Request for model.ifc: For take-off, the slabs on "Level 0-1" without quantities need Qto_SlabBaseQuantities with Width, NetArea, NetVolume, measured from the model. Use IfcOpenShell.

First a look at what the model holds.

```python
import ifcopenshell
import ifcopenshell.util.element
import ifcopenshell.util.unit

model = ifcopenshell.open("model.ifc")
print(model.schema)
for unit_type in ("LENGTHUNIT", "AREAUNIT", "VOLUMEUNIT"):
    print(unit_type, ifcopenshell.util.unit.calculate_unit_scale(model, unit_type))
storey = next(s for s in model.by_type("IfcBuildingStorey") if s.Name == "Level 0-1")
slabs = [e for e in ifcopenshell.util.element.get_decomposition(storey) if e.is_a("IfcSlab")]
for e in sorted(slabs, key=lambda e: e.id()):
    print(e.id(), e.is_a(), e.Name, list(ifcopenshell.util.element.get_psets(e, qtos_only=True)), sep=" | ")
```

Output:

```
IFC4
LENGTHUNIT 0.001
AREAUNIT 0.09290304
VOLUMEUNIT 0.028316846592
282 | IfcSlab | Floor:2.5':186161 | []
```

```python
import ifcopenshell
import ifcopenshell.api.pset
import ifcopenshell.geom
import ifcopenshell.util.element
import ifcopenshell.util.shape
import ifcopenshell.util.unit

model = ifcopenshell.open("model.ifc")
unit_scale = ifcopenshell.util.unit.calculate_unit_scale(model)
area_scale = ifcopenshell.util.unit.calculate_unit_scale(model, "AREAUNIT")
volume_scale = ifcopenshell.util.unit.calculate_unit_scale(model, "VOLUMEUNIT")
settings = ifcopenshell.geom.settings()

storey = next(s for s in model.by_type("IfcBuildingStorey") if s.Name == "Level 0-1")
slabs = [e for e in ifcopenshell.util.element.get_decomposition(storey) if e.is_a("IfcSlab")]

for e in sorted(slabs, key=lambda e: e.id()):
    if ifcopenshell.util.element.get_psets(e, qtos_only=True, should_inherit=False):
        continue
    # Geometry comes back in metres, in the element's own axes.
    shape = ifcopenshell.geom.create_shape(settings, e)
    values = {
        "Width": ifcopenshell.util.shape.get_z(shape.geometry) / unit_scale,
        "NetArea": ifcopenshell.util.shape.get_footprint_area(shape.geometry) / area_scale,
        "NetVolume": ifcopenshell.util.shape.get_volume(shape.geometry) / volume_scale,
    }
    qto = ifcopenshell.api.pset.add_qto(model, product=e, name="Qto_SlabBaseQuantities")
    ifcopenshell.api.pset.edit_qto(model, qto=qto, properties=values)
    print(e.id(), {k: round(v, 3) for k, v in values.items()})

model.write("model-out.ifc")
```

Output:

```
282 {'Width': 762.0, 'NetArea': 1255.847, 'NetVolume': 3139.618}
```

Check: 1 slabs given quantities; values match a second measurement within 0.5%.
